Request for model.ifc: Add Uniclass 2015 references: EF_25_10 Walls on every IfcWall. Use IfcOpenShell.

First a look at what the model holds.

```python
import ifcopenshell

model = ifcopenshell.open("model.ifc")
print(model.schema)
print("classifications:", [c.Name for c in model.by_type("IfcClassification")])
for ifc_class in ("IfcDoor", "IfcRoof", "IfcStair", "IfcWall", "IfcWindow"):
    print(ifc_class, len(model.by_type(ifc_class)))
```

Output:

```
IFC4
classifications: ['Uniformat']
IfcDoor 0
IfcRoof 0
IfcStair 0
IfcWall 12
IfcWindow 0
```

```python
import ifcopenshell
import ifcopenshell.api.classification

model = ifcopenshell.open("model.ifc")

system = ifcopenshell.api.classification.add_classification(model, classification="Uniclass 2015")

codes = {
    "IfcWall": ("EF_25_10", "Walls"),
}
for ifc_class, (code, name) in codes.items():
    products = model.by_type(ifc_class)
    ifcopenshell.api.classification.add_reference(
        model, products=products, classification=system, identification=code, name=name
    )
    print(code, len(products))

model.write("model_v2.ifc")
```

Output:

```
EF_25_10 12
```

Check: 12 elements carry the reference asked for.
